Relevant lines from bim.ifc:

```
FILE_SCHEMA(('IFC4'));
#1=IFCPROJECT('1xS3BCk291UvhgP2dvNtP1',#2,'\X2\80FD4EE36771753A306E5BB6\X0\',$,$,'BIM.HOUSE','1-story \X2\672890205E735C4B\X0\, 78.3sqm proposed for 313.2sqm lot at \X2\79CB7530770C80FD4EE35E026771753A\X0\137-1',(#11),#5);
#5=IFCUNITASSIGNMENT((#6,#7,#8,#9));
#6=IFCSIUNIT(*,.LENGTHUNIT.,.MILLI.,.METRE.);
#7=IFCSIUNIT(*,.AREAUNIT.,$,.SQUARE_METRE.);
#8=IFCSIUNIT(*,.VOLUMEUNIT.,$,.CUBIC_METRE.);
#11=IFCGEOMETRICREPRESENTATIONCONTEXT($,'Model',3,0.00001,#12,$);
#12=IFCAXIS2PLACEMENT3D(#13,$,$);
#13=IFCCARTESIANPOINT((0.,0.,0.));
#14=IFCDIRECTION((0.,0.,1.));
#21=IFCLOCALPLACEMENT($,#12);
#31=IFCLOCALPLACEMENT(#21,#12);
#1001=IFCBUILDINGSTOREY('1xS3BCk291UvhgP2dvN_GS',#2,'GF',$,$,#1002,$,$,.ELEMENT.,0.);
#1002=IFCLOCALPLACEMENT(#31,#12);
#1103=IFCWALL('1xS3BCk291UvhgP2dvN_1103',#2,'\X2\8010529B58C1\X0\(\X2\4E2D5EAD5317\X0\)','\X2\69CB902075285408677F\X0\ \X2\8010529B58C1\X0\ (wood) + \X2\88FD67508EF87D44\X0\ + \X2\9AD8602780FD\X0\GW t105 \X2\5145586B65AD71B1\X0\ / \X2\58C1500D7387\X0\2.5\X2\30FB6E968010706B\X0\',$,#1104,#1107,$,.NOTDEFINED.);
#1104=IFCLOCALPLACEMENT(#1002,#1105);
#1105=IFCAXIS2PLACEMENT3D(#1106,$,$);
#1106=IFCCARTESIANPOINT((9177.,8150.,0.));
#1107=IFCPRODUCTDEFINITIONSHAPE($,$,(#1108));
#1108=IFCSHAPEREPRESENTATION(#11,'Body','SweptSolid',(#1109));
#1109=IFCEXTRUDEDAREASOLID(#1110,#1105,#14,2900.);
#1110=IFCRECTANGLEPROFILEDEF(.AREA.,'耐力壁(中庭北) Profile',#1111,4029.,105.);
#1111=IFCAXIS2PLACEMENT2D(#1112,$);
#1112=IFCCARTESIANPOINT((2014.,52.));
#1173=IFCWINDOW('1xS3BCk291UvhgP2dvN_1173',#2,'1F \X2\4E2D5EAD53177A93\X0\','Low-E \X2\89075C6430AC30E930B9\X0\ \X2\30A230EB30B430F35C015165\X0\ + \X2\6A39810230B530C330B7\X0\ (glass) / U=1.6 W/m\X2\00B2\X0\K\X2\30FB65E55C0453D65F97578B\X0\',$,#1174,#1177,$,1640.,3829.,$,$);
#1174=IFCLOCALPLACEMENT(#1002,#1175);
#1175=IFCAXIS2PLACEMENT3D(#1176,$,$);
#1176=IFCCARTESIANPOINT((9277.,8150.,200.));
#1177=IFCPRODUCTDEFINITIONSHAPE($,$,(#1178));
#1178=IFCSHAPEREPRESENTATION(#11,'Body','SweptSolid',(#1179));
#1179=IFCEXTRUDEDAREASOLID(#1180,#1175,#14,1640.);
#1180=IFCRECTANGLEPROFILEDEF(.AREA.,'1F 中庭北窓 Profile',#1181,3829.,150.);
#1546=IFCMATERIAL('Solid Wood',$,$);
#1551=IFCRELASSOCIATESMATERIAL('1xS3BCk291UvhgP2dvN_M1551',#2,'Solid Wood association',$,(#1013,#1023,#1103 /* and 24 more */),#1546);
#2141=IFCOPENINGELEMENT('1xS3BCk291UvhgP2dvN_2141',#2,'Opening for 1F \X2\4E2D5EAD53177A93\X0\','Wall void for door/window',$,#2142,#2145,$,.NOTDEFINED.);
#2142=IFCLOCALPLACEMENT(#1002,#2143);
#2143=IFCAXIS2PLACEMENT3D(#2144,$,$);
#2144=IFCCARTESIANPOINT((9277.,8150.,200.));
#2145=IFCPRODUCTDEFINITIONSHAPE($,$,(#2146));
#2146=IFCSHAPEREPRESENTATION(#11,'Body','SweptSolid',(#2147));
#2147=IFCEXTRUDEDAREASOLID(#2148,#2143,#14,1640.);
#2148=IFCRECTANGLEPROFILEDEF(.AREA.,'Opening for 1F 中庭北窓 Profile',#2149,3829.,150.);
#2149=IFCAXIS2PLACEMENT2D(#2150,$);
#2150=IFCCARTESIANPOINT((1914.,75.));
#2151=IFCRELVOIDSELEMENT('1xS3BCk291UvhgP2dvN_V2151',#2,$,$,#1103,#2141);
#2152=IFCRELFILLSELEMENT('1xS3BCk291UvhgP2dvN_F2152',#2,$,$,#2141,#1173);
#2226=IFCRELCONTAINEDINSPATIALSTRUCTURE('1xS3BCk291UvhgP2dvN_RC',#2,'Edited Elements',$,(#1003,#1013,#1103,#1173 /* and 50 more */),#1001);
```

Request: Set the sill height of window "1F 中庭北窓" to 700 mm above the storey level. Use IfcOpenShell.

```python
import numpy as np
import ifcopenshell
import ifcopenshell.api.geometry
import ifcopenshell.geom
import ifcopenshell.util.element
import ifcopenshell.util.placement
import ifcopenshell.util.shape
import ifcopenshell.util.unit

model = ifcopenshell.open("bim.ifc")
unit_scale = ifcopenshell.util.unit.calculate_unit_scale(model)

window = model.by_id(1173)
opening = window.FillsVoids[0].RelatingOpeningElement
storey = ifcopenshell.util.element.get_container(window, ifc_class="IfcBuildingStorey")
level = ifcopenshell.util.placement.get_local_placement(storey.ObjectPlacement)[2, 3]

# The opening's origin need not be at the sill, so measure its lowest point.
shape = ifcopenshell.geom.create_shape(ifcopenshell.geom.settings(), opening)
bottom = ifcopenshell.util.shape.get_shape_bottom_elevation(shape, shape.geometry) / unit_scale
dz = level + 700.0 - bottom

shift = np.array([0.0, 0.0, dz])
# The window is not placed relative to its opening, so move both.
for product in (opening, window):
    matrix = ifcopenshell.util.placement.get_local_placement(product.ObjectPlacement)
    matrix[:3, 3] += shift
    ifcopenshell.api.geometry.edit_object_placement(model, product=product, matrix=matrix, is_si=False)

print(f"moved by {dz * unit_scale:+.3f} m")

model.write("bim_edited.ifc")
```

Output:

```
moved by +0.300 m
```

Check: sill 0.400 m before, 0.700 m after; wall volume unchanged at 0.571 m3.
